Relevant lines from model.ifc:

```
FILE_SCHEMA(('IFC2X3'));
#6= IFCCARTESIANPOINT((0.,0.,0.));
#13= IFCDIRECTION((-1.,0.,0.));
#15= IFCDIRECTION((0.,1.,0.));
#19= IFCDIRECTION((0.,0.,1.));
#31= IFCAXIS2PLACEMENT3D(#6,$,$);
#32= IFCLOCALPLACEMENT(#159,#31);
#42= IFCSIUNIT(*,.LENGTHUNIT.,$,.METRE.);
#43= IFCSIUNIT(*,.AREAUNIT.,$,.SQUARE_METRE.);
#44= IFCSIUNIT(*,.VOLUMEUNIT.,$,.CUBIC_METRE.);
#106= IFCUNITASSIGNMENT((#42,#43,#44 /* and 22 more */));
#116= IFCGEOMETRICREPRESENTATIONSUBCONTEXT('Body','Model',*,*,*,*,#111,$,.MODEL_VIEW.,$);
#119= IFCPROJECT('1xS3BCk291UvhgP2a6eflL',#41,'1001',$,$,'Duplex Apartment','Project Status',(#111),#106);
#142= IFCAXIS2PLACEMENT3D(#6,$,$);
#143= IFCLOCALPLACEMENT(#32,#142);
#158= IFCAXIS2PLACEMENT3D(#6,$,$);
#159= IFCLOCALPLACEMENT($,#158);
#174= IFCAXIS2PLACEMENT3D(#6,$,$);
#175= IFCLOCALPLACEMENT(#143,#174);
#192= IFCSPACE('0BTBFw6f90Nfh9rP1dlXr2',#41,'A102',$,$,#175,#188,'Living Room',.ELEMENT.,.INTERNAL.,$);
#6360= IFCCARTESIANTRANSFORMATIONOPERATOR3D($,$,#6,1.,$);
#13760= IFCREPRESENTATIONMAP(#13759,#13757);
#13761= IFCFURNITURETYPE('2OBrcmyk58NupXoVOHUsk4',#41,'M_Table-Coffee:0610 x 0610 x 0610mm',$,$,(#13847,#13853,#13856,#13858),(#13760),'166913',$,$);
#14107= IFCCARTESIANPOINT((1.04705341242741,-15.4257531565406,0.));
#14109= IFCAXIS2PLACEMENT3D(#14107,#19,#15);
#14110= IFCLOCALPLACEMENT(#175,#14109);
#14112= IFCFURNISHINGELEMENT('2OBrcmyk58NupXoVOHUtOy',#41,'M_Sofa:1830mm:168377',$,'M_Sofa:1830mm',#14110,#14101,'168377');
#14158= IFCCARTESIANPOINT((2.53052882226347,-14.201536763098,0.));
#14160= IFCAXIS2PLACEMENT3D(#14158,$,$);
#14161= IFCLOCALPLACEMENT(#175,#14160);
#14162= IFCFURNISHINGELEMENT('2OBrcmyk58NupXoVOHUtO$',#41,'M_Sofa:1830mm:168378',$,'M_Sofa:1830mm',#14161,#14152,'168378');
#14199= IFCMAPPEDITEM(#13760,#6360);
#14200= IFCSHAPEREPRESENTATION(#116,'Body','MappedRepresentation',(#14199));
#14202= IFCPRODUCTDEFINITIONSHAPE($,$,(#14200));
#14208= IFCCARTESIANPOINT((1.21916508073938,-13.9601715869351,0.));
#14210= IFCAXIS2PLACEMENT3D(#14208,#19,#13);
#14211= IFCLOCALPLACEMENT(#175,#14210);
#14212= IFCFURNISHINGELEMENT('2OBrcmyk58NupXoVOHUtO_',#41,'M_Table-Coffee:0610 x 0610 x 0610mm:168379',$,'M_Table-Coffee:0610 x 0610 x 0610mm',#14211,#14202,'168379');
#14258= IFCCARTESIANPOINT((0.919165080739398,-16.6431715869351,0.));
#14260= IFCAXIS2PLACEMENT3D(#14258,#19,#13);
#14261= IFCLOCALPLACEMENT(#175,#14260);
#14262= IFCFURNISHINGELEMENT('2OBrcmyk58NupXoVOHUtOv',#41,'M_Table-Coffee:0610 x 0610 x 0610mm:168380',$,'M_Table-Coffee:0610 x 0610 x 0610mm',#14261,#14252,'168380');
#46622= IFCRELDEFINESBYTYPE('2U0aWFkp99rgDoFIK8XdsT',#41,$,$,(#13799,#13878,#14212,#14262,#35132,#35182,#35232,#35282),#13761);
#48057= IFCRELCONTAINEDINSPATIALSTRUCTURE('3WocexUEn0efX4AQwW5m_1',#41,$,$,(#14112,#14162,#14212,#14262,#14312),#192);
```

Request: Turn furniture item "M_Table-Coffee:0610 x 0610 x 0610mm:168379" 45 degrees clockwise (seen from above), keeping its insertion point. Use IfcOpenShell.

```python
import ifcopenshell
import ifcopenshell.api.geometry
import ifcopenshell.util.placement

model = ifcopenshell.open("model.ifc")

item = model.by_guid("2OBrcmyk58NupXoVOHUtO_")
matrix = ifcopenshell.util.placement.get_local_placement(item.ObjectPlacement)
matrix = matrix @ ifcopenshell.util.placement.rotation(-45, "Z")
ifcopenshell.api.geometry.edit_object_placement(model, product=item, matrix=matrix, is_si=False)

print(ifcopenshell.util.placement.get_local_placement(item.ObjectPlacement).round(3) + 0.0)

model.write("model_edited.ifc")
```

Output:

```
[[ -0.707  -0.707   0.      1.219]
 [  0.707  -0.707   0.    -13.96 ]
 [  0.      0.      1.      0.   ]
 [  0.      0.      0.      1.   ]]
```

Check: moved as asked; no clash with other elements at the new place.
